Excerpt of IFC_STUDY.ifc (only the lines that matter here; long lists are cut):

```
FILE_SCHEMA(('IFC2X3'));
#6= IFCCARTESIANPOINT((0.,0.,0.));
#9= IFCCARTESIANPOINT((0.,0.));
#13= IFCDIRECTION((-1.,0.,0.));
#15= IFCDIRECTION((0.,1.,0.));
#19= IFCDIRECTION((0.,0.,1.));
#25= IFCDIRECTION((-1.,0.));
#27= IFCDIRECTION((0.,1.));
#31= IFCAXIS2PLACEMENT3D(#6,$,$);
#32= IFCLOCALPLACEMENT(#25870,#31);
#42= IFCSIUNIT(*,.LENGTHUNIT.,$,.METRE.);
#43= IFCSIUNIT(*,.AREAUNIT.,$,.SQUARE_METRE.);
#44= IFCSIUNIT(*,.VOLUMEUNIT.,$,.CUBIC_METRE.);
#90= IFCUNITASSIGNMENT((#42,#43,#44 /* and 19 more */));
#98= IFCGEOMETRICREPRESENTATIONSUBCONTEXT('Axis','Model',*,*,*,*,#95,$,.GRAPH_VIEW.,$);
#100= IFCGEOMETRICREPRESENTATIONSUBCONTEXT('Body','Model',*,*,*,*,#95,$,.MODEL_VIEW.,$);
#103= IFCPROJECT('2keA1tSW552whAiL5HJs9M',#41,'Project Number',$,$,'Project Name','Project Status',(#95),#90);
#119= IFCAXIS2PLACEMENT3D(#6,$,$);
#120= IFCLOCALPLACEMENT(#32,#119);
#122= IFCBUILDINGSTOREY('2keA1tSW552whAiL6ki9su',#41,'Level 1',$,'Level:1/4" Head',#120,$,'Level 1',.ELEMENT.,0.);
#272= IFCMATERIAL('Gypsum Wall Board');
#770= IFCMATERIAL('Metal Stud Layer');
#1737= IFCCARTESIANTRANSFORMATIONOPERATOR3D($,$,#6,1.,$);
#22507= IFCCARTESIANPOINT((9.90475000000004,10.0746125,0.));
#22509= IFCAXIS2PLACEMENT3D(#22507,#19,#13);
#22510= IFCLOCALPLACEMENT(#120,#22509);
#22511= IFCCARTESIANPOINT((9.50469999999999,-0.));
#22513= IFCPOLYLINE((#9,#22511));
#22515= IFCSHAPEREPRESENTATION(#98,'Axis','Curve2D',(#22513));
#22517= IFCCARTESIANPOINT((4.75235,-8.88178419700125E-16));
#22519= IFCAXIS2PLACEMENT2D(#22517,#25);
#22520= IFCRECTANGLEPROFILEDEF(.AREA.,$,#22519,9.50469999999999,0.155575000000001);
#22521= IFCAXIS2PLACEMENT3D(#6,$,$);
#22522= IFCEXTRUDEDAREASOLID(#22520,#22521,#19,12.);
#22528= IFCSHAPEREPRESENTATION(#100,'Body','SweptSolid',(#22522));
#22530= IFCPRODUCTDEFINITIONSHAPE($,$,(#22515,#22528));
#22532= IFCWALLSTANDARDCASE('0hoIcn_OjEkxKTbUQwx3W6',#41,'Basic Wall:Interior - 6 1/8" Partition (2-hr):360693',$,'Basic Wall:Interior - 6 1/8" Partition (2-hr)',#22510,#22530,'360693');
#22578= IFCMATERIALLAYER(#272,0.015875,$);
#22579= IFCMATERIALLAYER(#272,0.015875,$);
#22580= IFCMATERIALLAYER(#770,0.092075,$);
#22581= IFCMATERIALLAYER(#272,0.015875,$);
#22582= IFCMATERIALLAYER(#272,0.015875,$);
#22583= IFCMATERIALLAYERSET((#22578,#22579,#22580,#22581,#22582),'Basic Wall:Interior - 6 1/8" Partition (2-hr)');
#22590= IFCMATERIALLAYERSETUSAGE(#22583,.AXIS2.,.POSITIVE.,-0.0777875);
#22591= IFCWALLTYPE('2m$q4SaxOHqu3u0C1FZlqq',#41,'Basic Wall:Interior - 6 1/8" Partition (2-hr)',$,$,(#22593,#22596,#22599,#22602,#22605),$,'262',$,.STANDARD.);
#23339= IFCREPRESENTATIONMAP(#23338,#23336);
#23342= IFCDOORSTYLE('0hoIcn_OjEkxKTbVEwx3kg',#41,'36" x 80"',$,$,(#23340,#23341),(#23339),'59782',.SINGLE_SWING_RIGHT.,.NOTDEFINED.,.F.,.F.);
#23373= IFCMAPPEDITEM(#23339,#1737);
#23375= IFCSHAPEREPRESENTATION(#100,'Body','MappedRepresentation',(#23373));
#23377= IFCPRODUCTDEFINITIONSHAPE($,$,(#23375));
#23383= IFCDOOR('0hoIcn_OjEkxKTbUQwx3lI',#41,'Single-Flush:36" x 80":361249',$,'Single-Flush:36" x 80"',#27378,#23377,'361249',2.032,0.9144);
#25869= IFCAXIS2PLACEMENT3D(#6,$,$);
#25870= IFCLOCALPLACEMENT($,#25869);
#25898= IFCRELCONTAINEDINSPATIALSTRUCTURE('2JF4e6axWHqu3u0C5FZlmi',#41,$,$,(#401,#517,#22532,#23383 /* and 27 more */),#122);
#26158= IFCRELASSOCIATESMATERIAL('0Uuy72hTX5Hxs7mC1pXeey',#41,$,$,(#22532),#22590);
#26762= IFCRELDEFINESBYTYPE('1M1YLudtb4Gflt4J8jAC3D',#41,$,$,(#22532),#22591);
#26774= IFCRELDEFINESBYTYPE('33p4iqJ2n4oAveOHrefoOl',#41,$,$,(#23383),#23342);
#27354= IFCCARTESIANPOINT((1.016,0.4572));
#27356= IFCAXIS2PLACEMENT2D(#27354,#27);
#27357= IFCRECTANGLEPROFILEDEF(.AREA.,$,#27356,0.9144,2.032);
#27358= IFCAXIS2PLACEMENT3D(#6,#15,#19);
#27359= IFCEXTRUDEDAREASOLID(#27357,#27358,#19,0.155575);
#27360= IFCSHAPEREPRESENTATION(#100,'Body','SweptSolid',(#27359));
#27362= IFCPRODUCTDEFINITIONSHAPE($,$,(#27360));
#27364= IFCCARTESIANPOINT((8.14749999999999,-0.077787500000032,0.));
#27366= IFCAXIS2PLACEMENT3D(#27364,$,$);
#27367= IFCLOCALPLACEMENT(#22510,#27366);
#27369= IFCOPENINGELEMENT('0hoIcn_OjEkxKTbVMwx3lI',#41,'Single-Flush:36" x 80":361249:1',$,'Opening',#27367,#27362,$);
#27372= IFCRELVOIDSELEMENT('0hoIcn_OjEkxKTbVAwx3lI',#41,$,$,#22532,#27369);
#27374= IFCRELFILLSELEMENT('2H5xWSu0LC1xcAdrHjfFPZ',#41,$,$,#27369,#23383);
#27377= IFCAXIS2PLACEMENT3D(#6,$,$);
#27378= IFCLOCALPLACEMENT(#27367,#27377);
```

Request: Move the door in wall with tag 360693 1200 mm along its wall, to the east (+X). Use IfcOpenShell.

```python
import ifcopenshell
import ifcopenshell.api.geometry
import ifcopenshell.util.placement

model = ifcopenshell.open("IFC_STUDY.ifc")

door = model.by_guid("0hoIcn_OjEkxKTbUQwx3lI")
opening = door.FillsVoids[0].RelatingOpeningElement
wall = opening.VoidsElements[0].RelatingBuildingElement

wall_matrix = ifcopenshell.util.placement.get_local_placement(wall.ObjectPlacement)
shift = wall_matrix[:3, 0] * -1.2
before = ifcopenshell.util.placement.get_local_placement(door.ObjectPlacement)[:3, 3].copy()

# The door is placed relative to its opening, so it follows when the opening moves.
matrix = ifcopenshell.util.placement.get_local_placement(opening.ObjectPlacement)
matrix[:3, 3] += shift
ifcopenshell.api.geometry.edit_object_placement(
    model, product=opening, matrix=matrix, is_si=False, should_transform_children=True
)

after = ifcopenshell.util.placement.get_local_placement(door.ObjectPlacement)[:3, 3]
print("door moved by", (after - before).round(3) + 0.0)

model.write("IFC_STUDY_edited.ifc")
```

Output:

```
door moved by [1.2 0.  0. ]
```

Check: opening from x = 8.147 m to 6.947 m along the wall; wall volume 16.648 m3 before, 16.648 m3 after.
